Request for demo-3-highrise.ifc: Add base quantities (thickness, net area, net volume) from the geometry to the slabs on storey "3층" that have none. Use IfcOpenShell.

First a look at what the model holds.

```python
import ifcopenshell
import ifcopenshell.util.element
import ifcopenshell.util.unit

model = ifcopenshell.open("demo-3-highrise.ifc")
print(model.schema)
for unit_type in ("LENGTHUNIT", "AREAUNIT", "VOLUMEUNIT"):
    print(unit_type, ifcopenshell.util.unit.calculate_unit_scale(model, unit_type))
storey = next(s for s in model.by_type("IfcBuildingStorey") if s.Name == "3층")
slabs = [e for e in ifcopenshell.util.element.get_decomposition(storey) if e.is_a("IfcSlab")]
for e in sorted(slabs, key=lambda e: e.id()):
    print(e.id(), e.is_a(), e.Name, list(ifcopenshell.util.element.get_psets(e, qtos_only=True)), sep=" | ")
```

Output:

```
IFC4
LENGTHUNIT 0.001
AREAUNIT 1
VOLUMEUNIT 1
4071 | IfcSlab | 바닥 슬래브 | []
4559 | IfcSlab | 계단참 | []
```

```python
import ifcopenshell
import ifcopenshell.api.pset
import ifcopenshell.geom
import ifcopenshell.util.element
import ifcopenshell.util.shape
import ifcopenshell.util.unit

model = ifcopenshell.open("demo-3-highrise.ifc")
unit_scale = ifcopenshell.util.unit.calculate_unit_scale(model)
area_scale = ifcopenshell.util.unit.calculate_unit_scale(model, "AREAUNIT")
volume_scale = ifcopenshell.util.unit.calculate_unit_scale(model, "VOLUMEUNIT")
settings = ifcopenshell.geom.settings()

storey = next(s for s in model.by_type("IfcBuildingStorey") if s.Name == "3층")
slabs = [e for e in ifcopenshell.util.element.get_decomposition(storey) if e.is_a("IfcSlab")]

for e in sorted(slabs, key=lambda e: e.id()):
    if ifcopenshell.util.element.get_psets(e, qtos_only=True, should_inherit=False):
        continue
    # Geometry comes back in metres, in the element's own axes.
    shape = ifcopenshell.geom.create_shape(settings, e)
    values = {
        "Width": ifcopenshell.util.shape.get_z(shape.geometry) / unit_scale,
        "NetArea": ifcopenshell.util.shape.get_footprint_area(shape.geometry) / area_scale,
        "NetVolume": ifcopenshell.util.shape.get_volume(shape.geometry) / volume_scale,
    }
    qto = ifcopenshell.api.pset.add_qto(model, product=e, name="Qto_SlabBaseQuantities")
    ifcopenshell.api.pset.edit_qto(model, qto=qto, properties=values)
    print(e.id(), {k: round(v, 3) for k, v in values.items()})

model.write("demo-3-highrise_updated.ifc")
```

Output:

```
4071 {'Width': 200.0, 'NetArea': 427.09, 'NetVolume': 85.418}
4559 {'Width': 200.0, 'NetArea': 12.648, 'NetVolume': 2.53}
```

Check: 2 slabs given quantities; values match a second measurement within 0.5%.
